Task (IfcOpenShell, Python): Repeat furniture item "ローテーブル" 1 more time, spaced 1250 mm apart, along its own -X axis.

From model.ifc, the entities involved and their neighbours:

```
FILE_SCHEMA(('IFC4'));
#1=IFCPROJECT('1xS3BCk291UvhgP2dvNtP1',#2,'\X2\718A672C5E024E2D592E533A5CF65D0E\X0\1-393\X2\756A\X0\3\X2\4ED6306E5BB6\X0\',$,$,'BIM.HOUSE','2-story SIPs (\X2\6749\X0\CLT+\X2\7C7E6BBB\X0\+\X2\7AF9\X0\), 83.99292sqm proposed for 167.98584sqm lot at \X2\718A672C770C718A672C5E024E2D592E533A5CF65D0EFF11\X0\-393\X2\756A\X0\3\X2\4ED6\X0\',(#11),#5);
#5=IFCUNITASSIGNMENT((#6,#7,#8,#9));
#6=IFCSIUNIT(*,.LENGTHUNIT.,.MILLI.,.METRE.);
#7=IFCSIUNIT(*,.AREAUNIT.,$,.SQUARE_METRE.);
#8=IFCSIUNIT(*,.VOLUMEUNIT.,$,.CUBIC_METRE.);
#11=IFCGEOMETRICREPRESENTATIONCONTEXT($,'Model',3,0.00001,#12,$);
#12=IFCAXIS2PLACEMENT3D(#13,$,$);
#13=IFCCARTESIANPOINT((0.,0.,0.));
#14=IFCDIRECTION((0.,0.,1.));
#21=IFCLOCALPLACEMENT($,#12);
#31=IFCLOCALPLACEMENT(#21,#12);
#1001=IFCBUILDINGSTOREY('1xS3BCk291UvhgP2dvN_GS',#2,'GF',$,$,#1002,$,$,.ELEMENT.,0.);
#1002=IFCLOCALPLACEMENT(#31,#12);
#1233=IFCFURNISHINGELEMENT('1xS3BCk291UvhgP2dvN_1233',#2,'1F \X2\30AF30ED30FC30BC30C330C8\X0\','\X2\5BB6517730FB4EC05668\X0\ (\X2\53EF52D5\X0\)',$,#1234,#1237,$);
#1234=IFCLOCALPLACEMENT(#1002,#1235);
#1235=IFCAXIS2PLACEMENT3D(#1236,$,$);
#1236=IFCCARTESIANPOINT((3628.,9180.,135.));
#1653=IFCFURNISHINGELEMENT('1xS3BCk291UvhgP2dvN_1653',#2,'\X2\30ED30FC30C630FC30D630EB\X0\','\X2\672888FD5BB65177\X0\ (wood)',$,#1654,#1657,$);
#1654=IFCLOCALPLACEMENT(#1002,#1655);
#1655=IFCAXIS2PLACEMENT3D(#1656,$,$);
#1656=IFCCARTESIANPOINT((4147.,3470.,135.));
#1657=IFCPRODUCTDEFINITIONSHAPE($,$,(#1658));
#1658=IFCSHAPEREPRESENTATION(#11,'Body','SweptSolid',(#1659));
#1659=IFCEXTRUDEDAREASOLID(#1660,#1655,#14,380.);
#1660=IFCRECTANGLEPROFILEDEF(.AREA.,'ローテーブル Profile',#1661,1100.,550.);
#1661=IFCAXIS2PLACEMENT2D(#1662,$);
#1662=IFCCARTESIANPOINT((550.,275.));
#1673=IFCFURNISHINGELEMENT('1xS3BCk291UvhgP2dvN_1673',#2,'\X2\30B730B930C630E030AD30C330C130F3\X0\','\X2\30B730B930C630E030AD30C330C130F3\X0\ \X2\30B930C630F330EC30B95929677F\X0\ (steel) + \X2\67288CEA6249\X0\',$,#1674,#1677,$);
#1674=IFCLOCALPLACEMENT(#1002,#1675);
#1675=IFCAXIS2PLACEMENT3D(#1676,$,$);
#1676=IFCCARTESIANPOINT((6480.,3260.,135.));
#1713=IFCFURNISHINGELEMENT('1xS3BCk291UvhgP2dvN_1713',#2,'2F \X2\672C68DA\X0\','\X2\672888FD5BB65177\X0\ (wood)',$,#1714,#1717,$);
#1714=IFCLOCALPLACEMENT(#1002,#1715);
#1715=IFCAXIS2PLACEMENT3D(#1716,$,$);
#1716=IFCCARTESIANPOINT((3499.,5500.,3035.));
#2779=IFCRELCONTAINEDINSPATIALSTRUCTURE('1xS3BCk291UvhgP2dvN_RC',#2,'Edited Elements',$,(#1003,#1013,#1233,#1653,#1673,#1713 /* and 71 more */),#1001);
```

```python
import ifcopenshell
import ifcopenshell.api.geometry
import ifcopenshell.api.root
import ifcopenshell.util.element
import ifcopenshell.util.placement

model = ifcopenshell.open("model.ifc")


def reuse_history(source, copy):
    """copy_class also copies each property set's owner history, people and application; keep the originals."""
    for rel in copy.IsDefinedBy:
        if rel.is_a("IfcRelDefinesByProperties") and (history := rel.RelatingPropertyDefinition.OwnerHistory):
            rel.RelatingPropertyDefinition.OwnerHistory = source.OwnerHistory
            ifcopenshell.util.element.remove_deep2(model, history)


source = model.by_id(1653)
base = ifcopenshell.util.placement.get_local_placement(source.ObjectPlacement)
step = -base[:3, 0] * 1250.0

for i in range(1, 2):
    copy = ifcopenshell.api.root.copy_class(model, product=source)
    copy.Representation = ifcopenshell.util.element.copy_deep(
        model, source.Representation, exclude=["IfcGeometricRepresentationContext", "IfcRepresentationMap"]
    )
    reuse_history(source, copy)
    matrix = base.copy()
    matrix[:3, 3] += i * step
    print("added at", matrix[:3, 3].round(3) + 0.0)
    ifcopenshell.api.geometry.edit_object_placement(model, product=copy, matrix=matrix, is_si=False)

model.write("model_edited.ifc")
```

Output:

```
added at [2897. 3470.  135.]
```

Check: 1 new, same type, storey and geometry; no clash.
